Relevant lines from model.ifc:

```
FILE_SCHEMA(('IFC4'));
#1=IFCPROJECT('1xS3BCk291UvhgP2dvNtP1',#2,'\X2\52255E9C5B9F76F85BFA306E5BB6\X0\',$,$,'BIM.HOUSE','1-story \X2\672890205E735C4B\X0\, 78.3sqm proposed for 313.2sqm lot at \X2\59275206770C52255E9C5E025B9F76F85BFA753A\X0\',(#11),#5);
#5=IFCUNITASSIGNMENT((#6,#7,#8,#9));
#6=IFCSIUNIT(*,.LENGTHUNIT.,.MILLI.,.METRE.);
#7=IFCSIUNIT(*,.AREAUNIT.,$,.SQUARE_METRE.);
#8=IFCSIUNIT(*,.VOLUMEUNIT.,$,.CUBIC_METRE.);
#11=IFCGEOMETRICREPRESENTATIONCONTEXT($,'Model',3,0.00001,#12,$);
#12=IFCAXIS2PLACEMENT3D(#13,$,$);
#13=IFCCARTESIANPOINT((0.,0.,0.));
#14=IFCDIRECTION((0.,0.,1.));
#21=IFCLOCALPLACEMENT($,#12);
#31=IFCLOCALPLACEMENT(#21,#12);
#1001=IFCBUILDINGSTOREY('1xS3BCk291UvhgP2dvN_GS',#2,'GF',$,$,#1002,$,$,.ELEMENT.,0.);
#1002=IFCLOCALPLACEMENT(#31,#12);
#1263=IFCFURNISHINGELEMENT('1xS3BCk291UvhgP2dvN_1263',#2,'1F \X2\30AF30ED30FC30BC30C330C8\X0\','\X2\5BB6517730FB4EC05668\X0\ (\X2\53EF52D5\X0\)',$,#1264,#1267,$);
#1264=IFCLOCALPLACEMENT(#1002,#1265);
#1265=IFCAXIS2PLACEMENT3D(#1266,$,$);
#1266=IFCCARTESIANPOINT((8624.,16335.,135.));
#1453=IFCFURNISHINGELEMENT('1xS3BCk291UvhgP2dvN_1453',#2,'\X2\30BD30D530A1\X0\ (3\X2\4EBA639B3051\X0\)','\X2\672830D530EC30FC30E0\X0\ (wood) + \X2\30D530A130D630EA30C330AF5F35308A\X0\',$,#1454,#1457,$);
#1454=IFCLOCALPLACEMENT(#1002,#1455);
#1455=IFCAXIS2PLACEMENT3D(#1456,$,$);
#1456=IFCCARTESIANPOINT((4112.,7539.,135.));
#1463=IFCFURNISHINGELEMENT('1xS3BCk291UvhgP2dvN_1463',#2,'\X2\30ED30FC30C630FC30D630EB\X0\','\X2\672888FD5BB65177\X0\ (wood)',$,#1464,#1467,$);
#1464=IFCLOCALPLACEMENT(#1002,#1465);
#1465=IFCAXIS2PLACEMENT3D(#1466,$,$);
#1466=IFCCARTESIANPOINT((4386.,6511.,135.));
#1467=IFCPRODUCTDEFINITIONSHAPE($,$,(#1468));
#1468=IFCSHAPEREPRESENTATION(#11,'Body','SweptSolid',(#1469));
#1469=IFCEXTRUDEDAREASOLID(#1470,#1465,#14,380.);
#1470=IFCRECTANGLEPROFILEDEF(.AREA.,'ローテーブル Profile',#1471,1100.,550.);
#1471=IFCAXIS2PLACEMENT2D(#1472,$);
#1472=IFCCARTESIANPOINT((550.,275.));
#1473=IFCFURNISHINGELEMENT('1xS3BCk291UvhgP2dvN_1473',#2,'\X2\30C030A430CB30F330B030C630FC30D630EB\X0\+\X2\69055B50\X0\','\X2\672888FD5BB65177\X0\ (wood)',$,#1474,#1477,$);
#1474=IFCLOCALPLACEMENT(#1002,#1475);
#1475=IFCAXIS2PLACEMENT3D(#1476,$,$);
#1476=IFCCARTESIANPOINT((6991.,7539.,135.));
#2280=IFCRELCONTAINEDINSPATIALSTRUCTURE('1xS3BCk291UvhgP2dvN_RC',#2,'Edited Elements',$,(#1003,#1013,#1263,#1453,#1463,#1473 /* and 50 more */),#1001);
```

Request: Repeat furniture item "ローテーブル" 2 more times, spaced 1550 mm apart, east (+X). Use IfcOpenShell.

```python
import numpy as np
import ifcopenshell
import ifcopenshell.api.geometry
import ifcopenshell.api.root
import ifcopenshell.util.element
import ifcopenshell.util.placement

model = ifcopenshell.open("model.ifc")


def reuse_history(source, copy):
    """copy_class also copies each property set's owner history, people and application; keep the originals."""
    for rel in copy.IsDefinedBy:
        if rel.is_a("IfcRelDefinesByProperties") and (history := rel.RelatingPropertyDefinition.OwnerHistory):
            rel.RelatingPropertyDefinition.OwnerHistory = source.OwnerHistory
            ifcopenshell.util.element.remove_deep2(model, history)


source = model.by_id(1463)
base = ifcopenshell.util.placement.get_local_placement(source.ObjectPlacement)
step = np.array([1.0, 0.0, 0.0]) * 1550.0

for i in range(1, 3):
    copy = ifcopenshell.api.root.copy_class(model, product=source)
    copy.Representation = ifcopenshell.util.element.copy_deep(
        model, source.Representation, exclude=["IfcGeometricRepresentationContext", "IfcRepresentationMap"]
    )
    reuse_history(source, copy)
    matrix = base.copy()
    matrix[:3, 3] += i * step
    print("added at", matrix[:3, 3].round(3) + 0.0)
    ifcopenshell.api.geometry.edit_object_placement(model, product=copy, matrix=matrix, is_si=False)

model.write("model_edited.ifc")
```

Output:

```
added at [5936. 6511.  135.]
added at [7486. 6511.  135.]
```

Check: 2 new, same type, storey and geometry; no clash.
